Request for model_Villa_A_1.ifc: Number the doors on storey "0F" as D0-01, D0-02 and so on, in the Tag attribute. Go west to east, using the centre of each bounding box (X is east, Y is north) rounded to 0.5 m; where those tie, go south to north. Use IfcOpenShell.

First a look at what the model holds.

```python
import ifcopenshell
import ifcopenshell.util.element
import ifcopenshell.util.placement

model = ifcopenshell.open("model_Villa_A_1.ifc")
print(model.schema)
storey = next(s for s in model.by_type("IfcBuildingStorey") if s.Name == "0F")
doors = [e for e in ifcopenshell.util.element.get_decomposition(storey) if e.is_a("IfcDoor")]
for e in sorted(doors, key=lambda e: e.id()):
    origin = ifcopenshell.util.placement.get_local_placement(e.ObjectPlacement)[:3, 3]
    print(e.id(), e.Tag, e.Name, origin.round(2) + 0.0, sep=" | ")
```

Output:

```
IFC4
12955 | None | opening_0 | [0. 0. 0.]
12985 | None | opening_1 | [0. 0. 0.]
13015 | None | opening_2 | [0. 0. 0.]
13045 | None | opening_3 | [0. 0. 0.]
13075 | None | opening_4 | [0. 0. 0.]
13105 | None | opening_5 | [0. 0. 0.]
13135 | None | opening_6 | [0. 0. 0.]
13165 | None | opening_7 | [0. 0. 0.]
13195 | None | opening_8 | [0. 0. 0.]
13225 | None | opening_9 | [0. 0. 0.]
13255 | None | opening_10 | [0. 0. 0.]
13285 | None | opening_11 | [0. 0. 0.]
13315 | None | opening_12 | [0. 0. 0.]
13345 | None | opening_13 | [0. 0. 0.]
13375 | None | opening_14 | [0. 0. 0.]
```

```python
import ifcopenshell
import ifcopenshell.geom
import ifcopenshell.util.element
import ifcopenshell.util.shape

model = ifcopenshell.open("model_Villa_A_1.ifc")
settings = ifcopenshell.geom.settings()
settings.set("use-world-coords", True)


def centre(element):
    shape = ifcopenshell.geom.create_shape(settings, element)
    return ifcopenshell.util.shape.get_bbox_centroid(shape.geometry)


storey = next(s for s in model.by_type("IfcBuildingStorey") if s.Name == "0F")
doors = [e for e in ifcopenshell.util.element.get_decomposition(storey) if e.is_a("IfcDoor")]

# Insertion points can sit at a corner or the storey origin, so sort by the geometry (in metres).
centres = {e: centre(e) for e in doors}
doors.sort(key=lambda e: (round(centres[e][0] / 0.5), centres[e][1]))

for i, e in enumerate(doors, start=1):
    number = f"D0-{i:02d}"
    e.Tag = number
    print(e.id(), number)

model.write("model_Villa_A_1_rev.ifc")
```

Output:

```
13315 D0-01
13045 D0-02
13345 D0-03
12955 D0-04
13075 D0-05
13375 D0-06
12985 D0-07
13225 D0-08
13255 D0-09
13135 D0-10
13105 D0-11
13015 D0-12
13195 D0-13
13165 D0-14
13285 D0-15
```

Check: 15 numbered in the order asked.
